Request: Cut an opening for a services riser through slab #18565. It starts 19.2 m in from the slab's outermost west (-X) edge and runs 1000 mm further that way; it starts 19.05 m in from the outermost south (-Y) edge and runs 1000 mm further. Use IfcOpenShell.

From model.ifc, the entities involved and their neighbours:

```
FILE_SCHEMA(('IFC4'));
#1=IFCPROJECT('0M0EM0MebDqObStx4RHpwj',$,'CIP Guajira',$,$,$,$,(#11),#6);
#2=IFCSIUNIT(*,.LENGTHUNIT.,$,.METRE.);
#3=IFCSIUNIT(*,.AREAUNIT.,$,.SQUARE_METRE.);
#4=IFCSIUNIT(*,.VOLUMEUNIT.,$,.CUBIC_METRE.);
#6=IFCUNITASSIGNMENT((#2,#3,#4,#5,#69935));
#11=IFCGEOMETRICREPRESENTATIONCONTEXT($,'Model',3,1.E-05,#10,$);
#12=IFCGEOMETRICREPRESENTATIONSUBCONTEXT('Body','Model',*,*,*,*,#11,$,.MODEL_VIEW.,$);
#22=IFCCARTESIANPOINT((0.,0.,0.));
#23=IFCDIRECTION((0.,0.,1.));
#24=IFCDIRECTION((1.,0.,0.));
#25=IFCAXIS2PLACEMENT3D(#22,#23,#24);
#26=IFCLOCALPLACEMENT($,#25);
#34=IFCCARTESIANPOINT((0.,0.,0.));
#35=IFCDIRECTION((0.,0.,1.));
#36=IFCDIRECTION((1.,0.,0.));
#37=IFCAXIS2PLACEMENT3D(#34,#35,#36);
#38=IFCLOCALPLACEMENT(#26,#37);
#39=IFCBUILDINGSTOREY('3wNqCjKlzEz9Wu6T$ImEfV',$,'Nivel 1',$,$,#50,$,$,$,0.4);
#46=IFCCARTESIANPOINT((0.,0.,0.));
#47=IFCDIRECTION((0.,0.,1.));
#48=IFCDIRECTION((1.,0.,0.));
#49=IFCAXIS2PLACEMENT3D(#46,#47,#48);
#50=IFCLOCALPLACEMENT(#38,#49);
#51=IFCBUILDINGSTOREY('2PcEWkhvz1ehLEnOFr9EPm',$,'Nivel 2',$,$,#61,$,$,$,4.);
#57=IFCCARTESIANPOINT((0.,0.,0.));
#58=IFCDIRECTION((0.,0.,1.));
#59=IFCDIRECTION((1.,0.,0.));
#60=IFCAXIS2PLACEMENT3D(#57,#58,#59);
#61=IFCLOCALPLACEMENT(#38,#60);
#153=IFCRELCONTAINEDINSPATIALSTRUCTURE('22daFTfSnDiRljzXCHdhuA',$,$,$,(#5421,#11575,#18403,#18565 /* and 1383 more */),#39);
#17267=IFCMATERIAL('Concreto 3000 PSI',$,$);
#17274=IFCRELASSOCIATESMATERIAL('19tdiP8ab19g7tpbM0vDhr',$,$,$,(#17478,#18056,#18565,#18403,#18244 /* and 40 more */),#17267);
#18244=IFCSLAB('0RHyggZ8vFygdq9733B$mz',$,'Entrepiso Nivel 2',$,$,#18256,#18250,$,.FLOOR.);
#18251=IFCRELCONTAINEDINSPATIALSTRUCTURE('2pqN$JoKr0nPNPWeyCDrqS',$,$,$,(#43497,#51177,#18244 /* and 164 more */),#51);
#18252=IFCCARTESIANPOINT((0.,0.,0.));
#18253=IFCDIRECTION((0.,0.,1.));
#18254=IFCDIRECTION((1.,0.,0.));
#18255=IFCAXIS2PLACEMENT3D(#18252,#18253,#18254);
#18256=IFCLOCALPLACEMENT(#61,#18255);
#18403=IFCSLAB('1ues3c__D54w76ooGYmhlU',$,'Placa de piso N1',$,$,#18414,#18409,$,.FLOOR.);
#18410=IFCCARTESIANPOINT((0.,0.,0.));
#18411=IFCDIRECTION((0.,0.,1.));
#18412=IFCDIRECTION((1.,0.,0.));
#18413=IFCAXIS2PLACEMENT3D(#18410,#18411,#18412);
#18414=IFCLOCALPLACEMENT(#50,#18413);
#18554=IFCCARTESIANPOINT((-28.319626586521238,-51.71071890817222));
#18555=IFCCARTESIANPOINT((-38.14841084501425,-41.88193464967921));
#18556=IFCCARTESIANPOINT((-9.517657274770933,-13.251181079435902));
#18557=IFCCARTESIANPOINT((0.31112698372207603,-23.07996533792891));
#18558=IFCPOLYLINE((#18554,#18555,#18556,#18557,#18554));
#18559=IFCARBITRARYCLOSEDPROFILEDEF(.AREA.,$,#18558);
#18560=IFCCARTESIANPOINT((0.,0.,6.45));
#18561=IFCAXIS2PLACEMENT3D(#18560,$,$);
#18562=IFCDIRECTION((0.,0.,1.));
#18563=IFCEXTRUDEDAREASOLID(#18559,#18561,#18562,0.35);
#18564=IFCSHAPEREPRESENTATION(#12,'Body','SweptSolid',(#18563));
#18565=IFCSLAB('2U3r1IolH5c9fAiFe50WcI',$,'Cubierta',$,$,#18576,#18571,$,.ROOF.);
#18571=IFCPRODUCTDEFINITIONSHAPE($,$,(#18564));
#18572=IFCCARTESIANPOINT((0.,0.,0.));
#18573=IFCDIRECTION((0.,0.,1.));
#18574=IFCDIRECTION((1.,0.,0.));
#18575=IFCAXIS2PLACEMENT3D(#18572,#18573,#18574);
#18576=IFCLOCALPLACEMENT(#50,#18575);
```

```python
import numpy as np
import ifcopenshell
import ifcopenshell.api.feature
import ifcopenshell.api.geometry
import ifcopenshell.api.root
import ifcopenshell.geom
import ifcopenshell.util.placement
import ifcopenshell.util.representation
import ifcopenshell.util.shape
import ifcopenshell.util.unit

model = ifcopenshell.open("model.ifc")
unit_scale = ifcopenshell.util.unit.calculate_unit_scale(model)
settings = ifcopenshell.geom.settings()


def volume(element):
    """Net volume in cubic metres, openings subtracted."""
    shape = ifcopenshell.geom.create_shape(settings, element)
    return ifcopenshell.util.shape.get_volume(shape.geometry)


slab = model.by_id(18565)
before = volume(slab)

# Extent in the slab's own axes, in metres. The edges named are its -X and -Y sides.
slab_shape = ifcopenshell.geom.create_shape(settings, slab)
vertices = ifcopenshell.util.shape.get_vertices(slab_shape.geometry)
x_min, y_min, bottom = vertices.min(axis=0)
top = vertices[:, 2].max()

opening = ifcopenshell.api.root.create_entity(model, ifc_class="IfcOpeningElement", name="Services riser opening", predefined_type="OPENING")
context = ifcopenshell.util.representation.get_context(model, "Model", "Body", "MODEL_VIEW")
width, depth = 1, 1
outline = [(0.0, 0.0), (width, 0.0), (width, depth), (0.0, depth), (0.0, 0.0)]
# Overshoot both faces by 50 mm so the cut is clean.
shape = ifcopenshell.api.geometry.add_slab_representation(
    model, context=context, depth=top - bottom + 0.1, polyline=outline
)
ifcopenshell.api.geometry.assign_representation(model, product=opening, representation=shape)

matrix = ifcopenshell.util.placement.get_local_placement(slab.ObjectPlacement)
matrix[:, 3] = matrix @ np.append(np.array([x_min + 19.2, y_min + 19.05, bottom - 0.05]) / unit_scale, 1.0)
ifcopenshell.api.geometry.edit_object_placement(model, product=opening, matrix=matrix, is_si=False)
ifcopenshell.api.feature.add_feature(model, feature=opening, element=slab)

after = volume(slab)

print(f"slab volume {before:.3f} -> {after:.3f} m3")

model.write("model_v2.ifc")
```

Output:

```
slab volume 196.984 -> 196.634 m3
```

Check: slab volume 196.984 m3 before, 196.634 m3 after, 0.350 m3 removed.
